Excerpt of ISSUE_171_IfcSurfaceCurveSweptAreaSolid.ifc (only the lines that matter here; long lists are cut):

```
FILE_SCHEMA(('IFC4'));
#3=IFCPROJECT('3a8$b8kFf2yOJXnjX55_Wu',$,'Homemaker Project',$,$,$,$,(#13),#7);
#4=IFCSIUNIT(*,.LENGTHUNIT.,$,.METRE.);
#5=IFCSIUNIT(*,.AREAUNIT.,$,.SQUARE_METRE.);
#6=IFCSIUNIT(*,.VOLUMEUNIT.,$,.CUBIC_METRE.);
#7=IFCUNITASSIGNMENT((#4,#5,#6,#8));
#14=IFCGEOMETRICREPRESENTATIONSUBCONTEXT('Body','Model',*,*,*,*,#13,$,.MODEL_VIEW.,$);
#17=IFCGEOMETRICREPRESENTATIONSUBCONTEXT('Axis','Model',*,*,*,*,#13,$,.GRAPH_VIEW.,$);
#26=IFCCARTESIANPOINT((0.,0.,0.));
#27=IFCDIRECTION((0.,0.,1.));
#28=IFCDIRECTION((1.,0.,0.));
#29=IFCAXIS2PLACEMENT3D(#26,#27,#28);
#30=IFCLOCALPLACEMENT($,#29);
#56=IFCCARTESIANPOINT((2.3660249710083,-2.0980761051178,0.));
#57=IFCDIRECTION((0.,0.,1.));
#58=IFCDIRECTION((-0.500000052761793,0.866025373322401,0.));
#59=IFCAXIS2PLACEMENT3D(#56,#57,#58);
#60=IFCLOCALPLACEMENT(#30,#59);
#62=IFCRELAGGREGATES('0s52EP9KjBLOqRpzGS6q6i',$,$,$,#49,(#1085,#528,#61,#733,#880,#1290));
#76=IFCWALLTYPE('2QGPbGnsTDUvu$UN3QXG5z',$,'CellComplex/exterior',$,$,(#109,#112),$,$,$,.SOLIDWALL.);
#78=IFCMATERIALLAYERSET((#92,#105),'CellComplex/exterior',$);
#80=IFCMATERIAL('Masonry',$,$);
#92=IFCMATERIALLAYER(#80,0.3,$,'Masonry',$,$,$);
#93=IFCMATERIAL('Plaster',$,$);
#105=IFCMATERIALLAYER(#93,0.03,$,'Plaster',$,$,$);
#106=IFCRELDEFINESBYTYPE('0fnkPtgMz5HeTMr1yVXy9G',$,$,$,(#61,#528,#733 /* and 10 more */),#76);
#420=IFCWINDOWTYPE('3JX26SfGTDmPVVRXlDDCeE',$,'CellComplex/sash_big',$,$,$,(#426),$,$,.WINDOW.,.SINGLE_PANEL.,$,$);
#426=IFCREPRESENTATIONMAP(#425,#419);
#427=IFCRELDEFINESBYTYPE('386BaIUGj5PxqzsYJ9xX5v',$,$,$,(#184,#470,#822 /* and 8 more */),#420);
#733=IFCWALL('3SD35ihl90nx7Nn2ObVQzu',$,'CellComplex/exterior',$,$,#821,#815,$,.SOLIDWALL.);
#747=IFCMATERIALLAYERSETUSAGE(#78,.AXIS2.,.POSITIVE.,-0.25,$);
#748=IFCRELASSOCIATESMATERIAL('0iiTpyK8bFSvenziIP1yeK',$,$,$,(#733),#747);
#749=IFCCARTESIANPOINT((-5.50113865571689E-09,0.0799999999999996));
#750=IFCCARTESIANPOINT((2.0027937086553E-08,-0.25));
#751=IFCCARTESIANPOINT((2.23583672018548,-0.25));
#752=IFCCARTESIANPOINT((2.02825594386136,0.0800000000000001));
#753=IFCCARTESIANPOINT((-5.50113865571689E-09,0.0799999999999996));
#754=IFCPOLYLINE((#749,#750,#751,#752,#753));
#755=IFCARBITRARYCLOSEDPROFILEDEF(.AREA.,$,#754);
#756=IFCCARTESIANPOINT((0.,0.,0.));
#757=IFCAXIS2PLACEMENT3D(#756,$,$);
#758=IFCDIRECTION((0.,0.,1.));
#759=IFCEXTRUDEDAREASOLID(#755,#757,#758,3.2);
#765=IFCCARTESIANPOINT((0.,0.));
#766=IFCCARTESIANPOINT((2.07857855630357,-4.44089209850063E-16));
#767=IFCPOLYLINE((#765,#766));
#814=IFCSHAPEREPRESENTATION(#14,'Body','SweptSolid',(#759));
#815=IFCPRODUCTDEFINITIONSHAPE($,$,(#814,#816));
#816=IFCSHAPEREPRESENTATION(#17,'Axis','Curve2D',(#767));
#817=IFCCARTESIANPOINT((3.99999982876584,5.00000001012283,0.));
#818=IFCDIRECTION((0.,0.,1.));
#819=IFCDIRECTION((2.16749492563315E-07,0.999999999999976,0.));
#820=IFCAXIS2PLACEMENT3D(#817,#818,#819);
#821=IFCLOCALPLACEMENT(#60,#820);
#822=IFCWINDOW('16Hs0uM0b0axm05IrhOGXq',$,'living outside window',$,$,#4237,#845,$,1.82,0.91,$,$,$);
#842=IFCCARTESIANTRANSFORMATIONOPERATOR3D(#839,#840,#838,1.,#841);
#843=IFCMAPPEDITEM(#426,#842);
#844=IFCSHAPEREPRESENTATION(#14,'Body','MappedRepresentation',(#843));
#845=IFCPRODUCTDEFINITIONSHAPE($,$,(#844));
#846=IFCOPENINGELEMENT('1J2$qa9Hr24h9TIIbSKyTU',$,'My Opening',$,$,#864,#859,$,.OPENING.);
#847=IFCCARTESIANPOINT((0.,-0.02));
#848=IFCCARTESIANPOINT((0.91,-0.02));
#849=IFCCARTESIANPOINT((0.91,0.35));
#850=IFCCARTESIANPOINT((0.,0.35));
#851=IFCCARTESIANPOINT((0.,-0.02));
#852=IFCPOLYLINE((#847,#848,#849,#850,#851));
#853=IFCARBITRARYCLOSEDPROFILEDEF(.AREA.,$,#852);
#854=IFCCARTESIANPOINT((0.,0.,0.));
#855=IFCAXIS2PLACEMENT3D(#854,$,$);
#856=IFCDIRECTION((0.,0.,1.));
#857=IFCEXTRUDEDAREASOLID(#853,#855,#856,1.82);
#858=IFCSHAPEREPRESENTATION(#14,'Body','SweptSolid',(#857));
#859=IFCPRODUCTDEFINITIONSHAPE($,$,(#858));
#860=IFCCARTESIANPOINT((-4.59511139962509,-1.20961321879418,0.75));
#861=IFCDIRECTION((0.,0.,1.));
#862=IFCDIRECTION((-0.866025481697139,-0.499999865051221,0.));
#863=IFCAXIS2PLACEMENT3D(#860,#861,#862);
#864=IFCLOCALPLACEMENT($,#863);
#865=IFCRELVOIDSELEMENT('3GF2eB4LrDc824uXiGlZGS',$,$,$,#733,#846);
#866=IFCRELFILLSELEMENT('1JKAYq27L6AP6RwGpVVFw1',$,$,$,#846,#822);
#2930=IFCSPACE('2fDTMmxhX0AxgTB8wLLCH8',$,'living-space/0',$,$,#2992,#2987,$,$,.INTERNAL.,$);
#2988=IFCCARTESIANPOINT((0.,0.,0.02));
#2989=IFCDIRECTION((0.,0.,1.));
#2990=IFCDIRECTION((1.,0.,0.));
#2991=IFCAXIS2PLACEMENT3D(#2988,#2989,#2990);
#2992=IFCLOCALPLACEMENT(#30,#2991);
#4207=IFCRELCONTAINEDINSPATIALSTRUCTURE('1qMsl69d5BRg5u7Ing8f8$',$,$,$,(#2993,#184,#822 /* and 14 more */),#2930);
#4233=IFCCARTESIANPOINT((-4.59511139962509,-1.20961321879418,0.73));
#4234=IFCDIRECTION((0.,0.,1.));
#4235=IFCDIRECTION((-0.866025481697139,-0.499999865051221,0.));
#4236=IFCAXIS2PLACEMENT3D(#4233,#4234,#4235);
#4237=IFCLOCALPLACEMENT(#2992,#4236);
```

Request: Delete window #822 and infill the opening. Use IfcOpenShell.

```python
import ifcopenshell
import ifcopenshell.api.feature
import ifcopenshell.api.root
import ifcopenshell.geom
import ifcopenshell.util.shape

model = ifcopenshell.open("ISSUE_171_IfcSurfaceCurveSweptAreaSolid.ifc")
settings = ifcopenshell.geom.settings()


def volume(element):
    """Net volume in cubic metres, openings subtracted."""
    shape = ifcopenshell.geom.create_shape(settings, element)
    return ifcopenshell.util.shape.get_volume(shape.geometry)


window = model.by_guid("16Hs0uM0b0axm05IrhOGXq")
opening = window.FillsVoids[0].RelatingOpeningElement
wall = opening.VoidsElements[0].RelatingBuildingElement
before = volume(wall)

ifcopenshell.api.root.remove_product(model, product=window)
ifcopenshell.api.feature.remove_feature(model, feature=opening)

after = volume(wall)

print(f"wall volume {before:.3f} -> {after:.3f} m3")

model.write("ISSUE_171_IfcSurfaceCurveSweptAreaSolid_edited.ifc")
```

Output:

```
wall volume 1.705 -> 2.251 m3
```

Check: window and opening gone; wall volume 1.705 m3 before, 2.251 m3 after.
